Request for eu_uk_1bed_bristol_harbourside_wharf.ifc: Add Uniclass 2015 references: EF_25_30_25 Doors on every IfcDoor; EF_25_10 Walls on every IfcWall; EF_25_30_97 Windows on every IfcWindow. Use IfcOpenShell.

First a look at what the model holds.

```python
import ifcopenshell

model = ifcopenshell.open("eu_uk_1bed_bristol_harbourside_wharf.ifc")
print(model.schema)
print("classifications:", [c.Name for c in model.by_type("IfcClassification")])
for ifc_class in ("IfcDoor", "IfcRoof", "IfcStair", "IfcWall", "IfcWindow"):
    print(ifc_class, len(model.by_type(ifc_class)))
```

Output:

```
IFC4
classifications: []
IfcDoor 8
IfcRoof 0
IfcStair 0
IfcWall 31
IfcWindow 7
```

```python
import ifcopenshell
import ifcopenshell.api.classification

model = ifcopenshell.open("eu_uk_1bed_bristol_harbourside_wharf.ifc")

system = ifcopenshell.api.classification.add_classification(model, classification="Uniclass 2015")

codes = {
    "IfcDoor": ("EF_25_30_25", "Doors"),
    "IfcWall": ("EF_25_10", "Walls"),
    "IfcWindow": ("EF_25_30_97", "Windows"),
}
for ifc_class, (code, name) in codes.items():
    products = model.by_type(ifc_class)
    ifcopenshell.api.classification.add_reference(
        model, products=products, classification=system, identification=code, name=name
    )
    print(code, len(products))

model.write("eu_uk_1bed_bristol_harbourside_wharf_edited.ifc")
```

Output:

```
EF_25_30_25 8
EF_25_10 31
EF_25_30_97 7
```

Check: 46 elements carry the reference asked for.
